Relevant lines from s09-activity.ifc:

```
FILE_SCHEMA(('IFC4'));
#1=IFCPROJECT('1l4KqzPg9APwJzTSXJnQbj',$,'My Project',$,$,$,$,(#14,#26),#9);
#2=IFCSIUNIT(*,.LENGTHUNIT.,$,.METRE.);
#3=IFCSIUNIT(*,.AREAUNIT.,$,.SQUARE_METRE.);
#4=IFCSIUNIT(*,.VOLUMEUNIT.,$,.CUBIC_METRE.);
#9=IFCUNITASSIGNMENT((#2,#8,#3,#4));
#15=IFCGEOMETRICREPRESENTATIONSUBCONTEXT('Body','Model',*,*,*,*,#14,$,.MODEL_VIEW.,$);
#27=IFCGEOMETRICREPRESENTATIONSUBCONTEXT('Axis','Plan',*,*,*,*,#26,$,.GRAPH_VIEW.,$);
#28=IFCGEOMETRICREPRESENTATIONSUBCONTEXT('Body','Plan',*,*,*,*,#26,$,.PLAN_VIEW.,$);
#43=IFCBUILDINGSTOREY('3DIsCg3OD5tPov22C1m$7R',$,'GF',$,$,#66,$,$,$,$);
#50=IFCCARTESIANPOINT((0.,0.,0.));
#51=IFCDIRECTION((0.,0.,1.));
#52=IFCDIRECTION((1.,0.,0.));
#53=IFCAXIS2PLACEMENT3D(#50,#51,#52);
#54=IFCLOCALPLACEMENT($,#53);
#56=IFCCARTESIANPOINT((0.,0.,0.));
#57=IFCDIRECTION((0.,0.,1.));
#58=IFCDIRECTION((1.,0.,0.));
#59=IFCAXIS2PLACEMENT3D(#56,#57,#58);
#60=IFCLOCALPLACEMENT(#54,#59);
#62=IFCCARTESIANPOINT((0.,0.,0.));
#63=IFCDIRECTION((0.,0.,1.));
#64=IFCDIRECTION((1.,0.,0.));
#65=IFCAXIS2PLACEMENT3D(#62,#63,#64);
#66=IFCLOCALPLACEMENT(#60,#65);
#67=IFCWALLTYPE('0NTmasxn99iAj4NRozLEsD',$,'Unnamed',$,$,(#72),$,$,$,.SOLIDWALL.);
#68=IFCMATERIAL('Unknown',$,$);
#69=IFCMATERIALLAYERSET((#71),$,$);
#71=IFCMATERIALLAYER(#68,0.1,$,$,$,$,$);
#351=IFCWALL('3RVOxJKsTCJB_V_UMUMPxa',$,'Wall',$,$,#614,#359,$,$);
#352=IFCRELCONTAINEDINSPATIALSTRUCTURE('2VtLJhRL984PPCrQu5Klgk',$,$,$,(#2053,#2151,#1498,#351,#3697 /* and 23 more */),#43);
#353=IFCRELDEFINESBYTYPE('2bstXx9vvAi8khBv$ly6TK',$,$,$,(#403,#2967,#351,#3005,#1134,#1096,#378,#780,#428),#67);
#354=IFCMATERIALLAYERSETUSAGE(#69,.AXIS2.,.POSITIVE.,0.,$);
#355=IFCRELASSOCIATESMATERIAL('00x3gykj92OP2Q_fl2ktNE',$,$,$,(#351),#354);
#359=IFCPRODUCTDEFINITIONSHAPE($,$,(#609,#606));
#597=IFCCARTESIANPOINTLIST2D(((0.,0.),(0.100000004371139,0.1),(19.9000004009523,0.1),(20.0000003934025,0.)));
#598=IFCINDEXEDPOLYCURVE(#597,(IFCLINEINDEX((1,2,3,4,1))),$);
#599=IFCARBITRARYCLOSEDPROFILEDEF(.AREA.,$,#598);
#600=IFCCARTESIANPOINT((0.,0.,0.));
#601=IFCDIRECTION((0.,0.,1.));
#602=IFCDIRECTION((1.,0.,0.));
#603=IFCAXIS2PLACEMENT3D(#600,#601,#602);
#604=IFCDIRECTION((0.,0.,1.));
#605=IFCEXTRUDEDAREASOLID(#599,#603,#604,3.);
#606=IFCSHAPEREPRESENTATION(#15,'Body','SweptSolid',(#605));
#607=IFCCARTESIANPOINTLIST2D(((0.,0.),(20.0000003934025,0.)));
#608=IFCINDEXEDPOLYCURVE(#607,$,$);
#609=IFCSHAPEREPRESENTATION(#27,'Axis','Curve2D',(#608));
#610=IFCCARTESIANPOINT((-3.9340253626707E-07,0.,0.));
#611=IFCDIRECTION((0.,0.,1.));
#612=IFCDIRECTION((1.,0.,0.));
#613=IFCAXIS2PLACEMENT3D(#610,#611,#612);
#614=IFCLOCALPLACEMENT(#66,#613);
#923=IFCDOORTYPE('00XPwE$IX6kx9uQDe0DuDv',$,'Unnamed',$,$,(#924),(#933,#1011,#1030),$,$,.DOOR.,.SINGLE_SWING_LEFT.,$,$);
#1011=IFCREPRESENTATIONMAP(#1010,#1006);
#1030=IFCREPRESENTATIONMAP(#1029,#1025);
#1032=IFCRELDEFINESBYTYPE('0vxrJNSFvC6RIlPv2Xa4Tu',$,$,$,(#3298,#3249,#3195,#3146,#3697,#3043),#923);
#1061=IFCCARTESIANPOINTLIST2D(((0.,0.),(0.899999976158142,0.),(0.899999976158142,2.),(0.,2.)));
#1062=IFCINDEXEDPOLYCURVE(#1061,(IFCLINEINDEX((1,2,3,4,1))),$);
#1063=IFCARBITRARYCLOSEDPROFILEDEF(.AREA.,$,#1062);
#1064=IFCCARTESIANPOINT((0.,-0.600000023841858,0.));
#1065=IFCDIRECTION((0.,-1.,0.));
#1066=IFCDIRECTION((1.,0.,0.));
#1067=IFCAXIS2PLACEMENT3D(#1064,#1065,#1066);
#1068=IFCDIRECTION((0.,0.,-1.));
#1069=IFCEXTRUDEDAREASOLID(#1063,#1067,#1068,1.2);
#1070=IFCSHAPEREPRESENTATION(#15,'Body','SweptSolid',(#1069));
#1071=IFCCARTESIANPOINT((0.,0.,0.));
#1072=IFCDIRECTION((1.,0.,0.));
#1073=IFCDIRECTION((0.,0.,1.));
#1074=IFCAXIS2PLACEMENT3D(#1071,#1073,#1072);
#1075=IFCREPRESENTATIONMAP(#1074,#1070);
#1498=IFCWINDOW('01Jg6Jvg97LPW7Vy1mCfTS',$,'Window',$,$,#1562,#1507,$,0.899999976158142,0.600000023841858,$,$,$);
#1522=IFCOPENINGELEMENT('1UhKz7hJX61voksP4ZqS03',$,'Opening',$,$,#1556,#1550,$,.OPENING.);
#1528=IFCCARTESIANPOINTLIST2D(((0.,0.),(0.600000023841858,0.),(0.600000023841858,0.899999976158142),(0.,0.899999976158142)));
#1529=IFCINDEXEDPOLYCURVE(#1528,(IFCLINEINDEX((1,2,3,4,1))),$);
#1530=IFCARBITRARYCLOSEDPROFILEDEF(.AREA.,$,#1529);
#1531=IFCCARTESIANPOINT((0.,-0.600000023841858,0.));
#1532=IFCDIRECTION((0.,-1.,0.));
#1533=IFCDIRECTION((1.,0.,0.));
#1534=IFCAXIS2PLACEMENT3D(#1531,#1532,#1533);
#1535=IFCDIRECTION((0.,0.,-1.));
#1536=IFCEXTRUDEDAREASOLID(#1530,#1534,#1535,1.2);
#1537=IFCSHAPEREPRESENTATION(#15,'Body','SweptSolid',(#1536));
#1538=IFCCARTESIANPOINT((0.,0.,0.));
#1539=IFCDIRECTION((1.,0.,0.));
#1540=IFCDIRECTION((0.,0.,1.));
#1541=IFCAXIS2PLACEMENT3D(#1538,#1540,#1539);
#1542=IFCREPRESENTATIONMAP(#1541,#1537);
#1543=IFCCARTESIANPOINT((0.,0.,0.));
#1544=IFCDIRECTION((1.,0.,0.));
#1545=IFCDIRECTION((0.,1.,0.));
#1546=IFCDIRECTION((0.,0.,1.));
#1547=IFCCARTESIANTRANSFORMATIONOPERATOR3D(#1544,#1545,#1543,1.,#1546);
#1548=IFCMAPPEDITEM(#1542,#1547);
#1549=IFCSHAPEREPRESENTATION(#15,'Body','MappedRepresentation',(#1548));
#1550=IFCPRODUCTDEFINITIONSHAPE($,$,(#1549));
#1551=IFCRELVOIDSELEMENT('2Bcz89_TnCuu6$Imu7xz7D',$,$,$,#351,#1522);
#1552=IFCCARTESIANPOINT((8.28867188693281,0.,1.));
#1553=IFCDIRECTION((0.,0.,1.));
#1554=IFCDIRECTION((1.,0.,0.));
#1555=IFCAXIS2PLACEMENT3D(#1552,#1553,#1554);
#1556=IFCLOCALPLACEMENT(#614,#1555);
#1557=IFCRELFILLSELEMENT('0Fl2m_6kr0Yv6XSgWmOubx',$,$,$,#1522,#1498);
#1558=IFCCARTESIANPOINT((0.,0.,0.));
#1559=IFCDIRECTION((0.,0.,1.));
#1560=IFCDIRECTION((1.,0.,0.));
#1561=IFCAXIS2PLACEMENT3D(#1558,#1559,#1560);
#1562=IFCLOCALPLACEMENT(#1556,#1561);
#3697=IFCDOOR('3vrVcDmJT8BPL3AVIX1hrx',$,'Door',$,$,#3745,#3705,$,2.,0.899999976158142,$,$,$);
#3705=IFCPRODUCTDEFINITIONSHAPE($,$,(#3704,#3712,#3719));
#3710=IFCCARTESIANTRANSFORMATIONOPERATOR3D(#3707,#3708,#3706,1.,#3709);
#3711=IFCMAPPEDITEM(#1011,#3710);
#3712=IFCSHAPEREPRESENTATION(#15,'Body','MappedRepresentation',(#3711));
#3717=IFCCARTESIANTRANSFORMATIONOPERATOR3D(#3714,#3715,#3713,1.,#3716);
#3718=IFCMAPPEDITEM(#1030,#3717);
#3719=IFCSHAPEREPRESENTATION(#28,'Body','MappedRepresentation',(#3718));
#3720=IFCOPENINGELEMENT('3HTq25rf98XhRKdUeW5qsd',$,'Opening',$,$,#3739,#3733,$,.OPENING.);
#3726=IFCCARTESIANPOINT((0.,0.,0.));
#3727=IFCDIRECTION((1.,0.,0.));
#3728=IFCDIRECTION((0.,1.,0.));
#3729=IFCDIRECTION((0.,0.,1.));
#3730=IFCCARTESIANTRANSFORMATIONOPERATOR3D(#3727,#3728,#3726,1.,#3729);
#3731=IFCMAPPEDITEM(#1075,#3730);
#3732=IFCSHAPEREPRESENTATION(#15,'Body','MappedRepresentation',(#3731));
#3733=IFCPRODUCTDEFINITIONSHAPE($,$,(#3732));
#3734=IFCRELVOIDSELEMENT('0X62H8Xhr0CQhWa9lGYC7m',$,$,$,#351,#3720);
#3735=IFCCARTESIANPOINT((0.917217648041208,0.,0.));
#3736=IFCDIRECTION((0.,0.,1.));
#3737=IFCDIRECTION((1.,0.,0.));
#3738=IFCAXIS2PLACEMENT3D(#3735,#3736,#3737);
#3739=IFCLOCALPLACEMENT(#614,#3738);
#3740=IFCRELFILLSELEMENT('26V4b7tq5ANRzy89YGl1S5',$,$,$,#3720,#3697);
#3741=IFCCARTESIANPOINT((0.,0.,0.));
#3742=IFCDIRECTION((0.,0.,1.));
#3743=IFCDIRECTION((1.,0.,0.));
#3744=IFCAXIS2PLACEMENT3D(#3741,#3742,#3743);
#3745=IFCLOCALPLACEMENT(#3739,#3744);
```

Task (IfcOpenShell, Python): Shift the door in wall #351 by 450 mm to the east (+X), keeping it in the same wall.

```python
import ifcopenshell
import ifcopenshell.api.geometry
import ifcopenshell.util.placement
import ifcopenshell.util.unit

model = ifcopenshell.open("s09-activity.ifc")
unit_scale = ifcopenshell.util.unit.calculate_unit_scale(model)

door = model.by_guid("3vrVcDmJT8BPL3AVIX1hrx")
opening = door.FillsVoids[0].RelatingOpeningElement
wall = opening.VoidsElements[0].RelatingBuildingElement

wall_matrix = ifcopenshell.util.placement.get_local_placement(wall.ObjectPlacement)
shift = wall_matrix[:3, 0] * 0.45 / unit_scale
before = ifcopenshell.util.placement.get_local_placement(door.ObjectPlacement)[:3, 3].copy()

# The door is placed relative to its opening, so it follows when the opening moves.
matrix = ifcopenshell.util.placement.get_local_placement(opening.ObjectPlacement)
matrix[:3, 3] += shift
ifcopenshell.api.geometry.edit_object_placement(
    model, product=opening, matrix=matrix, is_si=False, should_transform_children=True
)

after = ifcopenshell.util.placement.get_local_placement(door.ObjectPlacement)[:3, 3]
print("door moved by", (after - before).round(3) + 0.0)

model.write("s09-activity_edited.ifc")
```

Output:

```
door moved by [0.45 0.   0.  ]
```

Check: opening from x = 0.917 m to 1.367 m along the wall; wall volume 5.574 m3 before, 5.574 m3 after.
